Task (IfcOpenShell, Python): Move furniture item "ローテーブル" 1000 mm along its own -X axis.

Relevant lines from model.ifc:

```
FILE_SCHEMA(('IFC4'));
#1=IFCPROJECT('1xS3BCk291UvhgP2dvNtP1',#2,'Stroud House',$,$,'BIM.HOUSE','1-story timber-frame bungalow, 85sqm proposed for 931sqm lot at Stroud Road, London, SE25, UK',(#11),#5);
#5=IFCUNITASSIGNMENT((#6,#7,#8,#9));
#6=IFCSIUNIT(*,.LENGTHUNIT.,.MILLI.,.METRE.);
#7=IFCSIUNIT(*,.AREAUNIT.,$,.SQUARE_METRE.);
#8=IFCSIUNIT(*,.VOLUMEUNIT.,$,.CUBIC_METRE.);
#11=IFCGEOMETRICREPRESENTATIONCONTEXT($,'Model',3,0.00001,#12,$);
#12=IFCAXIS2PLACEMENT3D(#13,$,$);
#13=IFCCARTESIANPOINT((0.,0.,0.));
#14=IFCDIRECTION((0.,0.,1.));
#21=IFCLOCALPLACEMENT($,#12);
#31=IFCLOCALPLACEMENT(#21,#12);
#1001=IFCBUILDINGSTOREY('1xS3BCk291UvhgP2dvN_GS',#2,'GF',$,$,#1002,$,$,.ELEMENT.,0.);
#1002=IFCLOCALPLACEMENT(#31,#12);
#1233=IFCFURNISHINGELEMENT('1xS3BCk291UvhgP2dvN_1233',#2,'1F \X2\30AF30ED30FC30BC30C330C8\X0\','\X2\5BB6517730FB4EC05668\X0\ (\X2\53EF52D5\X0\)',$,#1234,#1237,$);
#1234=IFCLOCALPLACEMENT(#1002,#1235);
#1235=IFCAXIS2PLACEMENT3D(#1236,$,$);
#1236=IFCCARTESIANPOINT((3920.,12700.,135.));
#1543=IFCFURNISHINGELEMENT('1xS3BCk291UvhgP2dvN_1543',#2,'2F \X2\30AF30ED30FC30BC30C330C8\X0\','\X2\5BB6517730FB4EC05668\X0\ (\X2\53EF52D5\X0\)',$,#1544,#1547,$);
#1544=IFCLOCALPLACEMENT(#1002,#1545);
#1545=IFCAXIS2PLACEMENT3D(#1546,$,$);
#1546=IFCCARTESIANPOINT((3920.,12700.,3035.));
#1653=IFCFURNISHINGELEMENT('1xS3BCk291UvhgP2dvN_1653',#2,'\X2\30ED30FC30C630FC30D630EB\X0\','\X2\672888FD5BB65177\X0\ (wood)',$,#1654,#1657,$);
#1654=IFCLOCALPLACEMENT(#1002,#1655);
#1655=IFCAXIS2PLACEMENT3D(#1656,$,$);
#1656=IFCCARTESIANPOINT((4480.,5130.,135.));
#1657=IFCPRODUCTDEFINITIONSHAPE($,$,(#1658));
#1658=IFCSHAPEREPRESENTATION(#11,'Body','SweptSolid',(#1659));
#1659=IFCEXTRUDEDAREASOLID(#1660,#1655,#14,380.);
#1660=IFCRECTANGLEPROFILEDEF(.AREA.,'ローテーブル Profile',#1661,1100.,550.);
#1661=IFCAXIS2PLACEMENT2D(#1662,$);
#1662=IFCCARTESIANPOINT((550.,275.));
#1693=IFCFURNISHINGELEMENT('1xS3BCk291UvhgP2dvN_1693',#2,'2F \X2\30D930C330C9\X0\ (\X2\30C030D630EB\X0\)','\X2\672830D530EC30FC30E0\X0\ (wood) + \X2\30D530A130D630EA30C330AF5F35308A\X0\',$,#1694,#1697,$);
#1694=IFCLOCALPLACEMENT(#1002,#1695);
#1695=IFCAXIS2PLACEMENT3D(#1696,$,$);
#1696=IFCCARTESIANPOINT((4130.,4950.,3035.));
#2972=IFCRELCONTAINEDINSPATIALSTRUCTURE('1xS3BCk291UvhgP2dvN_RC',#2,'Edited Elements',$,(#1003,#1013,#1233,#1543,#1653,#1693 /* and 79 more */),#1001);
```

```python
import ifcopenshell
import ifcopenshell.api.geometry
import ifcopenshell.util.placement
import ifcopenshell.util.unit

model = ifcopenshell.open("model.ifc")
unit_scale = ifcopenshell.util.unit.calculate_unit_scale(model)

item = model.by_guid("1xS3BCk291UvhgP2dvN_1653")
matrix = ifcopenshell.util.placement.get_local_placement(item.ObjectPlacement)
matrix[:3, 3] -= matrix[:3, 0] * 1 / unit_scale
ifcopenshell.api.geometry.edit_object_placement(model, product=item, matrix=matrix, is_si=False)

print(ifcopenshell.util.placement.get_local_placement(item.ObjectPlacement).round(3) + 0.0)

model.write("model_updated.ifc")
```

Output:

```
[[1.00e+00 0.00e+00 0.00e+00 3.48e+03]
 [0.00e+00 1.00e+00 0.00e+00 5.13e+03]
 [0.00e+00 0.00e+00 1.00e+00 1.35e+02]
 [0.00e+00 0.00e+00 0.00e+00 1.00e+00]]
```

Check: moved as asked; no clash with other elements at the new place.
